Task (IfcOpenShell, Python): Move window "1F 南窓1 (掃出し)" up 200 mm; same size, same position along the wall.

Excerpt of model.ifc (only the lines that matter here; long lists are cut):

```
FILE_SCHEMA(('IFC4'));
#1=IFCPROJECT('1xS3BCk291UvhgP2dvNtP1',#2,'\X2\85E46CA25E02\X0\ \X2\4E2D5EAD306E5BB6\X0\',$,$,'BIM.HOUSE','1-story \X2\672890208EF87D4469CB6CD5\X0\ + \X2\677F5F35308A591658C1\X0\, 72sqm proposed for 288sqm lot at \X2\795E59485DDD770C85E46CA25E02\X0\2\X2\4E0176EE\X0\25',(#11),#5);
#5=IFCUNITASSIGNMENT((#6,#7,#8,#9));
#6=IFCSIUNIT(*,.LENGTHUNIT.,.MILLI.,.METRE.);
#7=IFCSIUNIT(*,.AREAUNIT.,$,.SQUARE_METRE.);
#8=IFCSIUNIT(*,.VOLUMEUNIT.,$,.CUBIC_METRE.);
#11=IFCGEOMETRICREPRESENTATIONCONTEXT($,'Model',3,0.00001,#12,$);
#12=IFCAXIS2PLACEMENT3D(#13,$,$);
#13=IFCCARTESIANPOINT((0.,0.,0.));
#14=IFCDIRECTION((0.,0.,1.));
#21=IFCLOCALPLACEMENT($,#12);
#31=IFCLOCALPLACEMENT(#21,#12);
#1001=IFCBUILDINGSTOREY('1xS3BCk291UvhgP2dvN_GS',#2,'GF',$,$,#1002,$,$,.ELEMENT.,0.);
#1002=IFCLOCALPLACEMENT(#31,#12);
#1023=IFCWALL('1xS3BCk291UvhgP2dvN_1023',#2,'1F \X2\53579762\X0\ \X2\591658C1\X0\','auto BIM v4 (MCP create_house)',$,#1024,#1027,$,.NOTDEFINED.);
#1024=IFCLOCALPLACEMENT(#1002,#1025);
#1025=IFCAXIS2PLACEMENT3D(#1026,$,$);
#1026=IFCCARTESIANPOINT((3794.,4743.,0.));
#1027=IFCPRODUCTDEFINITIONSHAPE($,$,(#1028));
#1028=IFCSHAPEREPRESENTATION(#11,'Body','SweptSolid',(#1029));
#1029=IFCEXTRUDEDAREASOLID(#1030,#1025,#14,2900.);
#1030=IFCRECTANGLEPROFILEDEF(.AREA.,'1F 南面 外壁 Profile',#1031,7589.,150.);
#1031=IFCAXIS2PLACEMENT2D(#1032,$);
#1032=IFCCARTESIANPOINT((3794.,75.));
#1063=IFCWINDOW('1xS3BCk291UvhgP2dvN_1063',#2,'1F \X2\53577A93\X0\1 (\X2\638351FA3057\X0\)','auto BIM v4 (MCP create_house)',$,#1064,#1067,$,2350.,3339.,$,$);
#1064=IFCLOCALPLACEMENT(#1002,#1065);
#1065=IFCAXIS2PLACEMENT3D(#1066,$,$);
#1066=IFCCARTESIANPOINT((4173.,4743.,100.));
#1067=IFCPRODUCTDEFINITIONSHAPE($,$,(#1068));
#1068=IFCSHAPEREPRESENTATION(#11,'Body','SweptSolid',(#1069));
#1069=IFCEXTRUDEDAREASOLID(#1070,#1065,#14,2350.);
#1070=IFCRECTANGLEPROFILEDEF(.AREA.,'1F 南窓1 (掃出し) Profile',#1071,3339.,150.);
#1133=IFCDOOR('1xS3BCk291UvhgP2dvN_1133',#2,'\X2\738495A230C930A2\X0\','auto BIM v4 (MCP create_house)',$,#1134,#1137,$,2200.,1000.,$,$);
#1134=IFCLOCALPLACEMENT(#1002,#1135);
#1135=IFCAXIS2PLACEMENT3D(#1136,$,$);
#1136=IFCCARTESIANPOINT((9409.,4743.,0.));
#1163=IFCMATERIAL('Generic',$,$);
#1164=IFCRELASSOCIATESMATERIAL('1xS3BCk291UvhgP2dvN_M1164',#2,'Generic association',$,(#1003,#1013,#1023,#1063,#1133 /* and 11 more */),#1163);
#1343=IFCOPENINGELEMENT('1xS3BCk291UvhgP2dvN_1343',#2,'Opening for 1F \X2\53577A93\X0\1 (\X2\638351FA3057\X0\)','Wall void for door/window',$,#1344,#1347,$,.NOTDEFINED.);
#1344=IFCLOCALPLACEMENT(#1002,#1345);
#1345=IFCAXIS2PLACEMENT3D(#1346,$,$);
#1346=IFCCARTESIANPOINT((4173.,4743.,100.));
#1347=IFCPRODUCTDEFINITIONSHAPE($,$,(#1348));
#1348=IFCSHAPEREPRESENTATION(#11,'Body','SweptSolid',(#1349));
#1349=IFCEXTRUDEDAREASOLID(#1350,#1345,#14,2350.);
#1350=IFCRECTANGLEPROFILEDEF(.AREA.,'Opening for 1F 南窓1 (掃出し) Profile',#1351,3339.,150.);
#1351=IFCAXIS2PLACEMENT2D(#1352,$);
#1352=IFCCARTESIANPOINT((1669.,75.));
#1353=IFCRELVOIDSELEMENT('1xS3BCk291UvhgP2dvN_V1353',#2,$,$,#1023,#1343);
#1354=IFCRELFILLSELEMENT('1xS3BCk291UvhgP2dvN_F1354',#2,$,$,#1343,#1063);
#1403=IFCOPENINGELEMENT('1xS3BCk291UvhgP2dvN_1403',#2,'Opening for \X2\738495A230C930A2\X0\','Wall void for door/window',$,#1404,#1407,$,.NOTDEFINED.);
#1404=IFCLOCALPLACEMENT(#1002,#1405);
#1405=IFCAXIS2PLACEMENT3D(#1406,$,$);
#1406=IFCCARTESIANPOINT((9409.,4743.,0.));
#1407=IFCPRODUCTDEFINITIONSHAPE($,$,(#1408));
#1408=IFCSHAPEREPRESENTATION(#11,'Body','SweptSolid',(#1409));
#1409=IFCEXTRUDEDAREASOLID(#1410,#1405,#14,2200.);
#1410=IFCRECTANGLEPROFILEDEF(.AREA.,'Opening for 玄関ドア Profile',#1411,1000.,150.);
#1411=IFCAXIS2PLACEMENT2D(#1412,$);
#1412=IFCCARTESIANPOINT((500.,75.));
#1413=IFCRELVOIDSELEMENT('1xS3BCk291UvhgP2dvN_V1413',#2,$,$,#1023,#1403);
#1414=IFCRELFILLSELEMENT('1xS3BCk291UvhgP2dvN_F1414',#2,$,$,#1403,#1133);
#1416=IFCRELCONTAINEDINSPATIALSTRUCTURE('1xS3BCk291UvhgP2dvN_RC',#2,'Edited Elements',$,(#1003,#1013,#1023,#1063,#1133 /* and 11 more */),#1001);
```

```python
import numpy as np
import ifcopenshell
import ifcopenshell.api.geometry
import ifcopenshell.util.placement
import ifcopenshell.util.unit

model = ifcopenshell.open("model.ifc")
unit_scale = ifcopenshell.util.unit.calculate_unit_scale(model)

window = model.by_guid("1xS3BCk291UvhgP2dvN_1063")
opening = window.FillsVoids[0].RelatingOpeningElement
dz = 0.2 / unit_scale

shift = np.array([0.0, 0.0, dz])
# The window is not placed relative to its opening, so move both.
for product in (opening, window):
    matrix = ifcopenshell.util.placement.get_local_placement(product.ObjectPlacement)
    matrix[:3, 3] += shift
    ifcopenshell.api.geometry.edit_object_placement(model, product=product, matrix=matrix, is_si=False)

print(f"moved by {dz * unit_scale:+.3f} m")

model.write("model_updated.ifc")
```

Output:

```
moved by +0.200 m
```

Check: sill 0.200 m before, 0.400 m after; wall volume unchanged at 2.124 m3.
